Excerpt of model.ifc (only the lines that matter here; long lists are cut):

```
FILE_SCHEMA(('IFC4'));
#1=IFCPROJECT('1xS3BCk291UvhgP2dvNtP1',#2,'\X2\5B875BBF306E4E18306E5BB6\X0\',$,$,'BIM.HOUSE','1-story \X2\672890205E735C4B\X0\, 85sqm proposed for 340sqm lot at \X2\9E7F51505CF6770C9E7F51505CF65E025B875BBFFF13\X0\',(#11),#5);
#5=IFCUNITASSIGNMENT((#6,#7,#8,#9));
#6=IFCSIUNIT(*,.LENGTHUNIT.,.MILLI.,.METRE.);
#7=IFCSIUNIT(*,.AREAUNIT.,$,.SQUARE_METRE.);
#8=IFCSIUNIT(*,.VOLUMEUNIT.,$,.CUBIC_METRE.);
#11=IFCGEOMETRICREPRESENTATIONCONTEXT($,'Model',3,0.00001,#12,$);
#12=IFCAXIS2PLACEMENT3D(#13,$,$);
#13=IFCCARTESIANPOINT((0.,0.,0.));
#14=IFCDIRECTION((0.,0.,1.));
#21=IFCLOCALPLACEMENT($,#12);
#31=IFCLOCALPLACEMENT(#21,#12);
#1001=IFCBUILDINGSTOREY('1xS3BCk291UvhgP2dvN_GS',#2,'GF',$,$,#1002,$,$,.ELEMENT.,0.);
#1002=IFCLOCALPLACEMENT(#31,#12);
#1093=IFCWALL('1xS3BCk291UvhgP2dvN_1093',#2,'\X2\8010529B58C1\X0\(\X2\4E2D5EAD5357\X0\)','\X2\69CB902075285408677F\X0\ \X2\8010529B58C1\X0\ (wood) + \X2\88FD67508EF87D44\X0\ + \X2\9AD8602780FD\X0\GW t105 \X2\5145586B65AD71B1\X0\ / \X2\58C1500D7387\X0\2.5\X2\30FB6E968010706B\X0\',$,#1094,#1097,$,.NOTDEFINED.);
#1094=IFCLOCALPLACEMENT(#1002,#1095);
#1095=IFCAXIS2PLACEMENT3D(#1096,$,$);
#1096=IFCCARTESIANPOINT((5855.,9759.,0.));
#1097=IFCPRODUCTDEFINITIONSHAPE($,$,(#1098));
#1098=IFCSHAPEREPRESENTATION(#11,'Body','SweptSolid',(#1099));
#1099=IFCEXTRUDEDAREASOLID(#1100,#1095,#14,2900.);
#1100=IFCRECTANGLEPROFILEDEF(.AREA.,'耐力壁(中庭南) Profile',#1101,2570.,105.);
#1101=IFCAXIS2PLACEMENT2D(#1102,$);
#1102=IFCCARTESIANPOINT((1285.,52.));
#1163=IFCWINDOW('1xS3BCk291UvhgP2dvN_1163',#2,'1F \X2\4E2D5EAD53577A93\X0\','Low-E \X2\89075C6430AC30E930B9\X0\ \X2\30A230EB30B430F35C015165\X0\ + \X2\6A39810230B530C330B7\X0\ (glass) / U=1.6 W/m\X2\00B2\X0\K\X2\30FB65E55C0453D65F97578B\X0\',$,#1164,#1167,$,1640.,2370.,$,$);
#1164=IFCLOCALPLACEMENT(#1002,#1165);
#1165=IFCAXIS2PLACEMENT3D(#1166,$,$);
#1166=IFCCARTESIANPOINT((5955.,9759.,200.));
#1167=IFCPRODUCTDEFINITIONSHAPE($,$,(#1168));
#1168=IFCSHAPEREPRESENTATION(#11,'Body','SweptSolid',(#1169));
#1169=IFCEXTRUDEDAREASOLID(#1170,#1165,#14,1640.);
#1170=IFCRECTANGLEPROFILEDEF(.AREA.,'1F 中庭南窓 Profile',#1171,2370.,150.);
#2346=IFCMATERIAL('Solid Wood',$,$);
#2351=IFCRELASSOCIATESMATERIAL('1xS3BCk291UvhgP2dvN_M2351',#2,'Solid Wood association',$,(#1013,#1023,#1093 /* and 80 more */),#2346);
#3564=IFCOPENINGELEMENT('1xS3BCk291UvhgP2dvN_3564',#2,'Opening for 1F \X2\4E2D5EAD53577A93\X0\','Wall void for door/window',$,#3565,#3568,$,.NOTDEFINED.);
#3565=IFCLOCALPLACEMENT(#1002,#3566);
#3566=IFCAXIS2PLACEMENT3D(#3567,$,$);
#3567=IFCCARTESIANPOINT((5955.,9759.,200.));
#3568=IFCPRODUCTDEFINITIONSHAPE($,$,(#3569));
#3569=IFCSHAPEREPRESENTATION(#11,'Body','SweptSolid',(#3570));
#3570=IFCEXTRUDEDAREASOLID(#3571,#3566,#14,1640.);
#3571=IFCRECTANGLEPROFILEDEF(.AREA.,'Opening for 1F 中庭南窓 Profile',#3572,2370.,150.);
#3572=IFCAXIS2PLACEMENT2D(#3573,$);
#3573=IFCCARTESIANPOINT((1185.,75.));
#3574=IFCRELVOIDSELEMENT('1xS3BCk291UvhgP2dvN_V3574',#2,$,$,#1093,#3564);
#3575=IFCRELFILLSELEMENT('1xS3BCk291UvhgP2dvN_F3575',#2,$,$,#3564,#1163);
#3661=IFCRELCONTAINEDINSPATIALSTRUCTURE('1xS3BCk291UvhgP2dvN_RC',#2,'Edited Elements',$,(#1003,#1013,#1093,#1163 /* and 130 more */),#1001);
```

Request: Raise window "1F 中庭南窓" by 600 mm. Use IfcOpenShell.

```python
import numpy as np
import ifcopenshell
import ifcopenshell.api.geometry
import ifcopenshell.util.placement
import ifcopenshell.util.unit

model = ifcopenshell.open("model.ifc")
unit_scale = ifcopenshell.util.unit.calculate_unit_scale(model)

window = model.by_guid("1xS3BCk291UvhgP2dvN_1163")
opening = window.FillsVoids[0].RelatingOpeningElement
dz = 0.6 / unit_scale

shift = np.array([0.0, 0.0, dz])
# The window is not placed relative to its opening, so move both.
for product in (opening, window):
    matrix = ifcopenshell.util.placement.get_local_placement(product.ObjectPlacement)
    matrix[:3, 3] += shift
    ifcopenshell.api.geometry.edit_object_placement(model, product=product, matrix=matrix, is_si=False)

print(f"moved by {dz * unit_scale:+.3f} m")

model.write("model_edited.ifc")
```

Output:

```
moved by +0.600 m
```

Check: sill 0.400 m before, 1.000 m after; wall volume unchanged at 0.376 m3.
